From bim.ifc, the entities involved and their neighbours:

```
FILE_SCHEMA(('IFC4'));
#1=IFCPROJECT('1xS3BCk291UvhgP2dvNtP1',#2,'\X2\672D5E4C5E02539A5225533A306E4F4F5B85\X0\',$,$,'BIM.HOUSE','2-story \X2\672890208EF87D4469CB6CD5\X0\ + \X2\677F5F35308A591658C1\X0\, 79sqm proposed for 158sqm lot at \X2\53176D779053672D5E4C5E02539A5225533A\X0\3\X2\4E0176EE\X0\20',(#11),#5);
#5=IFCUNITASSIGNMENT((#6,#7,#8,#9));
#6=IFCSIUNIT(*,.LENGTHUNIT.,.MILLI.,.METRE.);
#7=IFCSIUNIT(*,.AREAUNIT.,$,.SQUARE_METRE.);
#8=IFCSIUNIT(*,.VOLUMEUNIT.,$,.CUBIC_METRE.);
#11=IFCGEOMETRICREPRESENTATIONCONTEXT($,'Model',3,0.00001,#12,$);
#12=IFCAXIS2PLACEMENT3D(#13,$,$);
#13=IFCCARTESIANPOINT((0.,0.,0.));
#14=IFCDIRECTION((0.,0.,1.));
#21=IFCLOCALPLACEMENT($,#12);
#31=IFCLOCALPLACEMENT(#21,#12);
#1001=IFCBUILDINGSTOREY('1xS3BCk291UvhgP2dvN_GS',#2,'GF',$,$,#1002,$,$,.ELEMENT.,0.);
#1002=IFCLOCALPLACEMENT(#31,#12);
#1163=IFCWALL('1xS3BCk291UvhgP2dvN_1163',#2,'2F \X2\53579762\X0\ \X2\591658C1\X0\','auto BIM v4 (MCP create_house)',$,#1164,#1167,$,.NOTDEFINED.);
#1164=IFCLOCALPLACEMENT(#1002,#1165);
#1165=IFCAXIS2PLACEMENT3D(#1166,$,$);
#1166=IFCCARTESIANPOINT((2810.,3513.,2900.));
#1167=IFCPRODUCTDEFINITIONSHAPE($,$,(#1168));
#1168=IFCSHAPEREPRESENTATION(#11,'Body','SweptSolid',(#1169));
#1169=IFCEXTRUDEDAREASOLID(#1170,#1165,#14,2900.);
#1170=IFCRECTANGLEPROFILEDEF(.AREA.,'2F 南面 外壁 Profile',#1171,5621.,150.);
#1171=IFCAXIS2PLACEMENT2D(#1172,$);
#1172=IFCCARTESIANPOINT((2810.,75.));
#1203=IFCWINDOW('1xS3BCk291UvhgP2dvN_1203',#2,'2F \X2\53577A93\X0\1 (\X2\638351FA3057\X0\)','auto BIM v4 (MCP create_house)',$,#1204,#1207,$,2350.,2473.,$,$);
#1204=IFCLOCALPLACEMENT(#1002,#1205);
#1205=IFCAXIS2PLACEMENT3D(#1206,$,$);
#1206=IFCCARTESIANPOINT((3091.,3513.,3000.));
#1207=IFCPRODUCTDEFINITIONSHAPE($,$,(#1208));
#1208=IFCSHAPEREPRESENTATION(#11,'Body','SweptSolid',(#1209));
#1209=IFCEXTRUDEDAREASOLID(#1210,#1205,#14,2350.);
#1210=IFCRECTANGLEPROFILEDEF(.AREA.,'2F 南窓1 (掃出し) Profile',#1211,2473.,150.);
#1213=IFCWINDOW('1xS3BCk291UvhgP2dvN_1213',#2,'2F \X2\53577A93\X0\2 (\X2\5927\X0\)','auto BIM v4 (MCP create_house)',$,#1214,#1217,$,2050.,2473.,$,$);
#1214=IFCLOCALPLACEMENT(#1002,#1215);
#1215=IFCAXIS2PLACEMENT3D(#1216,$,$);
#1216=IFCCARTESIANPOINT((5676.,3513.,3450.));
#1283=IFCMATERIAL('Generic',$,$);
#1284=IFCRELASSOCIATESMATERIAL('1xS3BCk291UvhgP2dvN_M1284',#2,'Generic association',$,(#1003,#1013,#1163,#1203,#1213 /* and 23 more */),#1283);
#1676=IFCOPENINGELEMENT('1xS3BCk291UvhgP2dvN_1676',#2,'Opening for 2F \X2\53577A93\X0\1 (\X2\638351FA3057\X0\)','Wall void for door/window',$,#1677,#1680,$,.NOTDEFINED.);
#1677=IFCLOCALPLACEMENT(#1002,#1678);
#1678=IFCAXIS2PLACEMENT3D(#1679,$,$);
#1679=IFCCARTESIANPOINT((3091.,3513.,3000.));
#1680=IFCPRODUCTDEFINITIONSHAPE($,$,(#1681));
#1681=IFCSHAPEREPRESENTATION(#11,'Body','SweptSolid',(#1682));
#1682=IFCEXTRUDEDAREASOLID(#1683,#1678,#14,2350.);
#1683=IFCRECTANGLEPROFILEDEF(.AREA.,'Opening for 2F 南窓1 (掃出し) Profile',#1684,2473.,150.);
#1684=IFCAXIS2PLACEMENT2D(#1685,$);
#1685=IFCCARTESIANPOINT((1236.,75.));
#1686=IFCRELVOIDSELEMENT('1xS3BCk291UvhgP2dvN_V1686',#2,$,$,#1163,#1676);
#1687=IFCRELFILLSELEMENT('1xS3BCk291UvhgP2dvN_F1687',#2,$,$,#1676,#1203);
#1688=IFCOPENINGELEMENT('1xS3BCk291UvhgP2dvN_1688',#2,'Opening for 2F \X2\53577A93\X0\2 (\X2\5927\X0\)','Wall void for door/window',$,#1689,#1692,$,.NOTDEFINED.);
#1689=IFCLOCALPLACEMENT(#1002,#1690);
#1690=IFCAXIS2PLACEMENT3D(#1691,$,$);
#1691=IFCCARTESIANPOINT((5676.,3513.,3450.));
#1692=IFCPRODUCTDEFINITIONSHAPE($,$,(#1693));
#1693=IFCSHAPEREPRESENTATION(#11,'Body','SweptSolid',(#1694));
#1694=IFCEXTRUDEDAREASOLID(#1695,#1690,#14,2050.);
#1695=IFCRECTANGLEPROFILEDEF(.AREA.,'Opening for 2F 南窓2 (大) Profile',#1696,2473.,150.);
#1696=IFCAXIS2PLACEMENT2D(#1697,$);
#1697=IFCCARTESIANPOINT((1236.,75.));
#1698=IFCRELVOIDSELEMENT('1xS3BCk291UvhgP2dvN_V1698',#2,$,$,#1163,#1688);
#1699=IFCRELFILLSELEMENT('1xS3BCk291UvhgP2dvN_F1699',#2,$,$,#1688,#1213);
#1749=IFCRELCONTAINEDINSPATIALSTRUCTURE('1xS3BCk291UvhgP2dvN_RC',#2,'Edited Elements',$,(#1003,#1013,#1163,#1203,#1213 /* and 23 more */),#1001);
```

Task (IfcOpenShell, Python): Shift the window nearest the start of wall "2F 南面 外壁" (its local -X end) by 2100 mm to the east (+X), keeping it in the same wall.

```python
import ifcopenshell
import ifcopenshell.api.geometry
import ifcopenshell.util.placement
import ifcopenshell.util.unit

model = ifcopenshell.open("bim.ifc")
unit_scale = ifcopenshell.util.unit.calculate_unit_scale(model)

window = model.by_id(1203)
opening = window.FillsVoids[0].RelatingOpeningElement
wall = opening.VoidsElements[0].RelatingBuildingElement

wall_matrix = ifcopenshell.util.placement.get_local_placement(wall.ObjectPlacement)
shift = wall_matrix[:3, 0] * 2.1 / unit_scale
before = ifcopenshell.util.placement.get_local_placement(window.ObjectPlacement)[:3, 3].copy()

# The window is not placed relative to its opening, so move both.
for product in (opening, window):
    matrix = ifcopenshell.util.placement.get_local_placement(product.ObjectPlacement)
    matrix[:3, 3] += shift
    ifcopenshell.api.geometry.edit_object_placement(model, product=product, matrix=matrix, is_si=False)

after = ifcopenshell.util.placement.get_local_placement(window.ObjectPlacement)[:3, 3]
print("window moved by", (after - before).round(3) + 0.0)

model.write("bim_updated.ifc")
```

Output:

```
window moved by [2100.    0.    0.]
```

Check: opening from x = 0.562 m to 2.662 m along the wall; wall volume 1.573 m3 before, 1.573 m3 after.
